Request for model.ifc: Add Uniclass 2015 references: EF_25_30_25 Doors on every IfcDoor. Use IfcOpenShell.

First a look at what the model holds.

```python
import ifcopenshell

model = ifcopenshell.open("model.ifc")
print(model.schema)
print("classifications:", [c.Name for c in model.by_type("IfcClassification")])
for ifc_class in ("IfcDoor", "IfcRoof", "IfcStair", "IfcWall", "IfcWindow"):
    print(ifc_class, len(model.by_type(ifc_class)))
```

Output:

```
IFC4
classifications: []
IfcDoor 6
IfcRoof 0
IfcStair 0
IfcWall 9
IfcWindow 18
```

```python
import ifcopenshell
import ifcopenshell.api.classification

model = ifcopenshell.open("model.ifc")

system = ifcopenshell.api.classification.add_classification(model, classification="Uniclass 2015")

codes = {
    "IfcDoor": ("EF_25_30_25", "Doors"),
}
for ifc_class, (code, name) in codes.items():
    products = model.by_type(ifc_class)
    ifcopenshell.api.classification.add_reference(
        model, products=products, classification=system, identification=code, name=name
    )
    print(code, len(products))

model.write("model-out.ifc")
```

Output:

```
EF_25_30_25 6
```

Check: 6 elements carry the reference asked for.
